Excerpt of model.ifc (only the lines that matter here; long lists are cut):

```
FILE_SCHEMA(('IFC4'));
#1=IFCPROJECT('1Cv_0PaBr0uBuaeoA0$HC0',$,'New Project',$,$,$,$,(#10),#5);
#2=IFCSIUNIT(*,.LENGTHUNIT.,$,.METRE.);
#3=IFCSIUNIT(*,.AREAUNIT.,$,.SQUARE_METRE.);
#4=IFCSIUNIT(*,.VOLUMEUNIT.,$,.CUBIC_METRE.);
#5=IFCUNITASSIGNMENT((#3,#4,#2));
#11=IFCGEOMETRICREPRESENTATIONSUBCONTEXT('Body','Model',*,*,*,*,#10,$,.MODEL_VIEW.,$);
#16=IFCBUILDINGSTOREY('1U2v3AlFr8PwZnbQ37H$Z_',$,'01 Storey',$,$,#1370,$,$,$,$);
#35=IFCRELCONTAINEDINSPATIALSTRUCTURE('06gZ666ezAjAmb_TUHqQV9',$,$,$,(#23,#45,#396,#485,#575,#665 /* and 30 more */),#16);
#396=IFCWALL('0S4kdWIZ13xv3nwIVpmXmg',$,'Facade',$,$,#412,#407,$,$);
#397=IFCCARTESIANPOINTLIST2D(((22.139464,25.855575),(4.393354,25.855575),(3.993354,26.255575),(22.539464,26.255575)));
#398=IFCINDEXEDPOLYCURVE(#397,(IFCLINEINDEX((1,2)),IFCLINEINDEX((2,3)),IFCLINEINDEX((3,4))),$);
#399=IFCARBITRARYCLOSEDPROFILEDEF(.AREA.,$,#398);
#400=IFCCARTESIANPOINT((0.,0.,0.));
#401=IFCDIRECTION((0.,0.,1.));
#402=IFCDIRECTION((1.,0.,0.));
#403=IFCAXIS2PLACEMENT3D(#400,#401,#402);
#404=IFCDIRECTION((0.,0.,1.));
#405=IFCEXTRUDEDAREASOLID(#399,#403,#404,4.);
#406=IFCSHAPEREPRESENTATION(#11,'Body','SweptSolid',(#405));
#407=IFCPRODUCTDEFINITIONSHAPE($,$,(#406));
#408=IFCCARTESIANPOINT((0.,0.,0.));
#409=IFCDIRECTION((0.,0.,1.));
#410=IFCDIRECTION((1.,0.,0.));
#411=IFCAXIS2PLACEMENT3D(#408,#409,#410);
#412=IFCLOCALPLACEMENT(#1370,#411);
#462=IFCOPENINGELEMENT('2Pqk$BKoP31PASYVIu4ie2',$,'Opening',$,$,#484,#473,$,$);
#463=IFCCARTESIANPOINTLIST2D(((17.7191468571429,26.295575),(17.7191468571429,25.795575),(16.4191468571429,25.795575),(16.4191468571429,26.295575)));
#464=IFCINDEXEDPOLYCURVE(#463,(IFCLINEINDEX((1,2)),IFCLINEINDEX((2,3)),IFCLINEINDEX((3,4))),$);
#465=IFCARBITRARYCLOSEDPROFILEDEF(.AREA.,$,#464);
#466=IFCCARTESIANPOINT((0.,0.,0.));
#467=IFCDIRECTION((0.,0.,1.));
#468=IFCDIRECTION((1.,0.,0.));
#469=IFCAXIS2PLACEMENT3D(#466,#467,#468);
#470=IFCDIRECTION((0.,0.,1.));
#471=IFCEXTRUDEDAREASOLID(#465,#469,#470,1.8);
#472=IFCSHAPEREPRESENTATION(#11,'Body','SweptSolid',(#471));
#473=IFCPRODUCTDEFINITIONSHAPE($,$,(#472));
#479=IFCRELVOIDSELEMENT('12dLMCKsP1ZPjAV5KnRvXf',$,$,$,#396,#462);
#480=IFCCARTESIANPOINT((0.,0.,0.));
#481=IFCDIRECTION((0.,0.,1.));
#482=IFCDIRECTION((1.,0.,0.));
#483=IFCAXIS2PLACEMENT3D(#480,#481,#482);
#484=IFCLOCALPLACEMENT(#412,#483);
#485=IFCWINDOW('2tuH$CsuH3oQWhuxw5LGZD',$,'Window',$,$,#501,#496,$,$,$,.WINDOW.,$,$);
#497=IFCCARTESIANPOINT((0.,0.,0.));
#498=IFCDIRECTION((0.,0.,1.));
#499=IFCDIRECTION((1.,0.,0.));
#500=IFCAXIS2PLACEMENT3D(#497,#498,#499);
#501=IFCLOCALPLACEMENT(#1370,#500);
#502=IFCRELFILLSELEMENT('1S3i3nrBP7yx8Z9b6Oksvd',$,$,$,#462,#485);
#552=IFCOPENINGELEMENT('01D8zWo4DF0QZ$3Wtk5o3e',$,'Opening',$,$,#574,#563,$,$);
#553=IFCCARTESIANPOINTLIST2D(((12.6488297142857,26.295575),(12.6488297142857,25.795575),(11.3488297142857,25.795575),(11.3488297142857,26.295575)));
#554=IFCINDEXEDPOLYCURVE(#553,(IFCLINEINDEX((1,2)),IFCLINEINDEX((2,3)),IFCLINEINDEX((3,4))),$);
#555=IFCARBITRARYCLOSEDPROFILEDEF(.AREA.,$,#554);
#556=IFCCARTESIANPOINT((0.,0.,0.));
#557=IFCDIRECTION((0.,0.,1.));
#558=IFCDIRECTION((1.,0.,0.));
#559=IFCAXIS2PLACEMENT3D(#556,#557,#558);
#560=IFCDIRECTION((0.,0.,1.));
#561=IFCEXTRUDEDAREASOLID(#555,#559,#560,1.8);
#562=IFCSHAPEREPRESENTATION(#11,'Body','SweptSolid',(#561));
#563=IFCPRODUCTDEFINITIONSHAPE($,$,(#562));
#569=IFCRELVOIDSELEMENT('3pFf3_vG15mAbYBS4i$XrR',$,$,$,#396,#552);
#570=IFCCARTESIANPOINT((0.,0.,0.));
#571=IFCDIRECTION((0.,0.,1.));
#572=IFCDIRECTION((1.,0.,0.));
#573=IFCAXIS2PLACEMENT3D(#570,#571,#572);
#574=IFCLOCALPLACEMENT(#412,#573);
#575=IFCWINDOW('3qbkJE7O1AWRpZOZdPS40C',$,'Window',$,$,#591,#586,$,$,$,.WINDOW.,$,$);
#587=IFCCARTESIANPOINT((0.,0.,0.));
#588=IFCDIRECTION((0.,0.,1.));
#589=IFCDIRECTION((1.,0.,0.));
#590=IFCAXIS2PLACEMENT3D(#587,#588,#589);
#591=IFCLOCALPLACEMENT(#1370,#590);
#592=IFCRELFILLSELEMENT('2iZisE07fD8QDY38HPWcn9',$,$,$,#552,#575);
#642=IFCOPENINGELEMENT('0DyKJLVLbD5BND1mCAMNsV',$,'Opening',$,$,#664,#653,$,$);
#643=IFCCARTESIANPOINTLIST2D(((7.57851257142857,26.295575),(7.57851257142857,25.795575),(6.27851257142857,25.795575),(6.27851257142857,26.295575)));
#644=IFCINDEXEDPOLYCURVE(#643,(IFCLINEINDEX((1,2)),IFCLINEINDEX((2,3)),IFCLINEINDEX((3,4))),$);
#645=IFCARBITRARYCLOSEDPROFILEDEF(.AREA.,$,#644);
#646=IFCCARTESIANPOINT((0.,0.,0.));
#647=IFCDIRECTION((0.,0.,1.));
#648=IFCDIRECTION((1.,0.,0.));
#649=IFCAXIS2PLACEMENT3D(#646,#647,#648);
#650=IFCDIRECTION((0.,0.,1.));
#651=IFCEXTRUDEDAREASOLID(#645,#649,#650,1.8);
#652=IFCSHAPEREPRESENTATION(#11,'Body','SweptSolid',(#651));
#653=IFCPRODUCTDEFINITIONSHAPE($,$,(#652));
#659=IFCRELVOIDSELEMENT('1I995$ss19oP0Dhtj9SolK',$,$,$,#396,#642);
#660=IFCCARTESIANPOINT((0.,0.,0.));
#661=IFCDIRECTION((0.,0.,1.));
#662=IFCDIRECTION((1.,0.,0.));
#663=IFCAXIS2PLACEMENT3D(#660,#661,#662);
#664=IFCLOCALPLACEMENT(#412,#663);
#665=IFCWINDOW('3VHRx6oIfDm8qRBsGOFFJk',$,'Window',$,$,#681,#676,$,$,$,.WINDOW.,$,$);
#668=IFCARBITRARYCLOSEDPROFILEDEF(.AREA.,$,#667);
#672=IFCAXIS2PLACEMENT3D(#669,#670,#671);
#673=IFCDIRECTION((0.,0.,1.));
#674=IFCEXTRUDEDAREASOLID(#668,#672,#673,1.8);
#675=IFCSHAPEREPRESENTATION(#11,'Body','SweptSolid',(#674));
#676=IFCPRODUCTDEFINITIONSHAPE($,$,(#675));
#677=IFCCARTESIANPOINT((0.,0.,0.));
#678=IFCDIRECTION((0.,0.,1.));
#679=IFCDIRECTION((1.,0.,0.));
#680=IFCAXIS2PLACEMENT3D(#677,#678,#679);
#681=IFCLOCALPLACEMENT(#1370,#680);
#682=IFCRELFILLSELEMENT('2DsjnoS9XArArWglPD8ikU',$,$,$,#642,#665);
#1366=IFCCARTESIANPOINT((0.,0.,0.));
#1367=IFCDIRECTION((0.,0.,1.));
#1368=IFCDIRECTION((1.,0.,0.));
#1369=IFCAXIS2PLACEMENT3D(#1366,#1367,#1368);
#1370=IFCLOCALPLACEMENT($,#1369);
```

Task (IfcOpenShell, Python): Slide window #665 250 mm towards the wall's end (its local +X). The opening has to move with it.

```python
import ifcopenshell
import ifcopenshell.api.geometry
import ifcopenshell.util.placement
import ifcopenshell.util.unit

model = ifcopenshell.open("model.ifc")
unit_scale = ifcopenshell.util.unit.calculate_unit_scale(model)

window = model.by_id(665)
opening = window.FillsVoids[0].RelatingOpeningElement
wall = opening.VoidsElements[0].RelatingBuildingElement

wall_matrix = ifcopenshell.util.placement.get_local_placement(wall.ObjectPlacement)
shift = wall_matrix[:3, 0] * 0.25 / unit_scale
before = ifcopenshell.util.placement.get_local_placement(window.ObjectPlacement)[:3, 3].copy()

# The window is not placed relative to its opening, so move both.
for product in (opening, window):
    matrix = ifcopenshell.util.placement.get_local_placement(product.ObjectPlacement)
    matrix[:3, 3] += shift
    ifcopenshell.api.geometry.edit_object_placement(model, product=product, matrix=matrix, is_si=False)

after = ifcopenshell.util.placement.get_local_placement(window.ObjectPlacement)[:3, 3]
print("window moved by", (after - before).round(3) + 0.0)

model.write("model_v2.ifc")
```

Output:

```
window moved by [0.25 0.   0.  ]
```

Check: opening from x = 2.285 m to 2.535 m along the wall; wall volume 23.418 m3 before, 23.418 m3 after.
